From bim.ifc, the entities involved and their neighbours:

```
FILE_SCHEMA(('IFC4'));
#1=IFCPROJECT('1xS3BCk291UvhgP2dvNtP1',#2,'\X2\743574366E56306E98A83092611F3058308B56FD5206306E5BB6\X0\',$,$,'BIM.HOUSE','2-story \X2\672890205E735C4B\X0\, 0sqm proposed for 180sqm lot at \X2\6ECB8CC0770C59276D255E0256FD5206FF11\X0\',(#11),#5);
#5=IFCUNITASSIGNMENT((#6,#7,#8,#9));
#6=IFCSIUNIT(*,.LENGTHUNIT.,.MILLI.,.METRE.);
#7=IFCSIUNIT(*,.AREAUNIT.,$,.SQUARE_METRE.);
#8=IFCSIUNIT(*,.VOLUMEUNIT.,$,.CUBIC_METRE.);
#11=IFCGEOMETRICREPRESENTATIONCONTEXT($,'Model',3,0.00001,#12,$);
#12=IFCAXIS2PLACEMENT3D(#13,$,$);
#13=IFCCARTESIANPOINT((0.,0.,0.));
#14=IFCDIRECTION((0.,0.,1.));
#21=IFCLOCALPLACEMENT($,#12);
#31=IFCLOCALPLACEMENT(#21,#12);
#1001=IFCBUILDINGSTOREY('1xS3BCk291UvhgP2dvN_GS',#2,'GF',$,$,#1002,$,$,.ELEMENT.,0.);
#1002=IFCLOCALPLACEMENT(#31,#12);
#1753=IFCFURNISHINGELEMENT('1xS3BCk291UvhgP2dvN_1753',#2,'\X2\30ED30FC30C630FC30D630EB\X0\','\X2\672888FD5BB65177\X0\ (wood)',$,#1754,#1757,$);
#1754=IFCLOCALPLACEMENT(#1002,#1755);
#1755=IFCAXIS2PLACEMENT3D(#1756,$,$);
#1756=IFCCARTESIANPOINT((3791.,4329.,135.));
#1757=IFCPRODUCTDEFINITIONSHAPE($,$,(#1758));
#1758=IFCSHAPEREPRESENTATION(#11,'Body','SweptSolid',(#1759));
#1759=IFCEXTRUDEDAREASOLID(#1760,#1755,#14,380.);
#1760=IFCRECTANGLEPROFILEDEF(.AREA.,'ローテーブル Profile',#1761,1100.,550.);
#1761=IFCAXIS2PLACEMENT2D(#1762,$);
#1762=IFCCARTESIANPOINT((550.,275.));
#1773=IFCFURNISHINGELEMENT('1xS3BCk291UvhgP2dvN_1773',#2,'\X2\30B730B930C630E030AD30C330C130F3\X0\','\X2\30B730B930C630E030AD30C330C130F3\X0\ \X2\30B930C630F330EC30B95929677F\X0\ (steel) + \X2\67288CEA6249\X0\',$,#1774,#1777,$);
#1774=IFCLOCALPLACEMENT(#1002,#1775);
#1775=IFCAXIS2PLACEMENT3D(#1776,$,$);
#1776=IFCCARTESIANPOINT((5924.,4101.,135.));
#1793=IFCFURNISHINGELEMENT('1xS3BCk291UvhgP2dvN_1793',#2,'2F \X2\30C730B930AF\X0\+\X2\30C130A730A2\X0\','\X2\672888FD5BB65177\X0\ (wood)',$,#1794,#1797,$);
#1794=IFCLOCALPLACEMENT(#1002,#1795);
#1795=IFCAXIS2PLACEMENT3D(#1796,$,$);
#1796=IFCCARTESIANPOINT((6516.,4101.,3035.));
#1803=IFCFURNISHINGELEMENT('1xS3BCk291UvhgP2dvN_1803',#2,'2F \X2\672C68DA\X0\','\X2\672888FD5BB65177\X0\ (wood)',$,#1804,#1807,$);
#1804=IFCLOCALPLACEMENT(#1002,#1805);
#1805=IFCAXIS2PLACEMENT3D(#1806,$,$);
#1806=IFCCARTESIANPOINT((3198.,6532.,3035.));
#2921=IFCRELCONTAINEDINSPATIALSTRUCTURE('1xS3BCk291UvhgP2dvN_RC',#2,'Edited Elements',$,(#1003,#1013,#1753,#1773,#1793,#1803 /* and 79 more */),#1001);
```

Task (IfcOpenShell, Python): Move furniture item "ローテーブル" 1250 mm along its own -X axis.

```python
import ifcopenshell
import ifcopenshell.api.geometry
import ifcopenshell.util.placement
import ifcopenshell.util.unit

model = ifcopenshell.open("bim.ifc")
unit_scale = ifcopenshell.util.unit.calculate_unit_scale(model)

item = model.by_guid("1xS3BCk291UvhgP2dvN_1753")
matrix = ifcopenshell.util.placement.get_local_placement(item.ObjectPlacement)
matrix[:3, 3] -= matrix[:3, 0] * 1.25 / unit_scale
ifcopenshell.api.geometry.edit_object_placement(model, product=item, matrix=matrix, is_si=False)

print(ifcopenshell.util.placement.get_local_placement(item.ObjectPlacement).round(3) + 0.0)

model.write("bim_updated.ifc")
```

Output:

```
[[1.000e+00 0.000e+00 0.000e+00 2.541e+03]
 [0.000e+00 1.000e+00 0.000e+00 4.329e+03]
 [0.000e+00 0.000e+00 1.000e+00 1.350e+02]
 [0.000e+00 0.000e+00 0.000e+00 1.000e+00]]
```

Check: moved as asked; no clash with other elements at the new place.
